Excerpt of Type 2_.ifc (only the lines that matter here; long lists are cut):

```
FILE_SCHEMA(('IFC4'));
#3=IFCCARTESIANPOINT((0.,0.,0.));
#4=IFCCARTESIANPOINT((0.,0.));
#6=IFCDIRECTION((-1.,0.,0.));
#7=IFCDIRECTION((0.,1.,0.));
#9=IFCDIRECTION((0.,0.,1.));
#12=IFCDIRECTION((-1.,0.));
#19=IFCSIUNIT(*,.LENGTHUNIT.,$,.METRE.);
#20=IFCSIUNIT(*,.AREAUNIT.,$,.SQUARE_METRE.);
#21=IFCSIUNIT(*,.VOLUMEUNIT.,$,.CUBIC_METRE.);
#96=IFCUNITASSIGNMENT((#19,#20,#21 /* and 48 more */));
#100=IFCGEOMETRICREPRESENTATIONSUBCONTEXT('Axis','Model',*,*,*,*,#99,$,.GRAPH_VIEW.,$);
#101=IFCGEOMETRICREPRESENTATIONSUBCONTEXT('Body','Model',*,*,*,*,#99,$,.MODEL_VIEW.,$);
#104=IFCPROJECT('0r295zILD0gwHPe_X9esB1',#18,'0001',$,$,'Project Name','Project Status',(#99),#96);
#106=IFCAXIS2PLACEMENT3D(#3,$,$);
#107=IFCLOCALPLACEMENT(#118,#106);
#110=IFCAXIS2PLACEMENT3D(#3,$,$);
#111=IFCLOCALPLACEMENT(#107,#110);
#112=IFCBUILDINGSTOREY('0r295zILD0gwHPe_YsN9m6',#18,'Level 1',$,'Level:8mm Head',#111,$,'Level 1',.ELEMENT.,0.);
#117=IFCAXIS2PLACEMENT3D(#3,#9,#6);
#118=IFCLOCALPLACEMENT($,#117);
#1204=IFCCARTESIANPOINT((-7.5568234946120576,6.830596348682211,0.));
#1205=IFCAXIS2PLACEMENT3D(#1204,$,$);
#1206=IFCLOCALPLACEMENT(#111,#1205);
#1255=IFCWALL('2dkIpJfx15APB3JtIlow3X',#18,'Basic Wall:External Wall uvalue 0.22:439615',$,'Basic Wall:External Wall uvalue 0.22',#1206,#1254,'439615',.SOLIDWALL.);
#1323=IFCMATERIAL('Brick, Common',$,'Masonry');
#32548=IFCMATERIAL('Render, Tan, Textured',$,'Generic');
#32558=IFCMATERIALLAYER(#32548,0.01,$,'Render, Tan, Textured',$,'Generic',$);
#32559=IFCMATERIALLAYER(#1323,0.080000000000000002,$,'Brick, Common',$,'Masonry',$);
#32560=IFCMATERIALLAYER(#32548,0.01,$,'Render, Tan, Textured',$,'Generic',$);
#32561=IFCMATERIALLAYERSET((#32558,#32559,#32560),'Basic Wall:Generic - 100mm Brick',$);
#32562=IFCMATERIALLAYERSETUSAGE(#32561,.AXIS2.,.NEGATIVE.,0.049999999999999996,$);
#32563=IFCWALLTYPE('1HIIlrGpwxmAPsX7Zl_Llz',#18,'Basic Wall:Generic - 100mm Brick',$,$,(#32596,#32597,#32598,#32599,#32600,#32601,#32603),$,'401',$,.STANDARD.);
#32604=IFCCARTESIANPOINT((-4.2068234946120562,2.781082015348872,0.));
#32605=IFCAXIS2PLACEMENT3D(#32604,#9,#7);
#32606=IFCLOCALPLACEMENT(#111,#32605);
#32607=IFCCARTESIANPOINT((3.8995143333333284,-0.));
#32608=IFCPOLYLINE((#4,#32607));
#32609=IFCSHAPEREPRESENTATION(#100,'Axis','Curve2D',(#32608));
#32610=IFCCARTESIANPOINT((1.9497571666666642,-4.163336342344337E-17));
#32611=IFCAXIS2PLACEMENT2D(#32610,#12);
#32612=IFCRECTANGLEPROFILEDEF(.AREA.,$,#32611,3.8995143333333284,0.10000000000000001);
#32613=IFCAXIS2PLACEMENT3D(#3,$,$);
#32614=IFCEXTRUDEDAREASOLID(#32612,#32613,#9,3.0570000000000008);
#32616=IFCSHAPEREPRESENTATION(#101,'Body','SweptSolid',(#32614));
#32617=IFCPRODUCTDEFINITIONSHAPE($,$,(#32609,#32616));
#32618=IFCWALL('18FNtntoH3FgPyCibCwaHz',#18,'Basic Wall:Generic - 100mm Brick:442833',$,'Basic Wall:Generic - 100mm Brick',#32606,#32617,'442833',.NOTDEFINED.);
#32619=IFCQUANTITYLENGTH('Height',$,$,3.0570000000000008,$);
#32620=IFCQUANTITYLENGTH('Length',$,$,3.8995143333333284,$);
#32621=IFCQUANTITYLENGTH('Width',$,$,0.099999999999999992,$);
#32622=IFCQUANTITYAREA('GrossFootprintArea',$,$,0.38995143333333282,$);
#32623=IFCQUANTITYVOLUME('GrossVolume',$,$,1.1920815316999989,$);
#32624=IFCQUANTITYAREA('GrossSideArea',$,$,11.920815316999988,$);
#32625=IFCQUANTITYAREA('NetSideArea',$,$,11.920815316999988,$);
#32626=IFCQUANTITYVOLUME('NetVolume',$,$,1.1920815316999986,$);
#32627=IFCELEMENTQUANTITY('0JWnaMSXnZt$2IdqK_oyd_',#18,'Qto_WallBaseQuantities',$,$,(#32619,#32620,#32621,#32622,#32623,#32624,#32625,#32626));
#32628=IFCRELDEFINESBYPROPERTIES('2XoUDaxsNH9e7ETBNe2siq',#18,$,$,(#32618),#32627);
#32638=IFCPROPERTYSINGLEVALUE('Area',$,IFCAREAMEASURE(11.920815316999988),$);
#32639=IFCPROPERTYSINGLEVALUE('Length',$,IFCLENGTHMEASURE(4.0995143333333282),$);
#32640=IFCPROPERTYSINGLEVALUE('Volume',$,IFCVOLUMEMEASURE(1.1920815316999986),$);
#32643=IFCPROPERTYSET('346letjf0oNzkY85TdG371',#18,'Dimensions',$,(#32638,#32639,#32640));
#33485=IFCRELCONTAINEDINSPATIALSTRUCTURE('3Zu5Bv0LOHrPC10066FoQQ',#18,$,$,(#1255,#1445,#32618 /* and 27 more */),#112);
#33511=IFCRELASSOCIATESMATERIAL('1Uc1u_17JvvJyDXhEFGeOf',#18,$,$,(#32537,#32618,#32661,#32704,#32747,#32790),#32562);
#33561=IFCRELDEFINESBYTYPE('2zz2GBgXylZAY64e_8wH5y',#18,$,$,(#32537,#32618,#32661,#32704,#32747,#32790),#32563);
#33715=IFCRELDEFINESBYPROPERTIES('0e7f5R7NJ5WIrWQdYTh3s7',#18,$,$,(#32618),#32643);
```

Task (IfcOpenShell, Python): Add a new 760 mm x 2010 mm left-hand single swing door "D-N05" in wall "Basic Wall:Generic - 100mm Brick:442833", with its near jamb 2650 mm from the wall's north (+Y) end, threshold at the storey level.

```python
import numpy as np
import ifcopenshell
import ifcopenshell.api.feature
import ifcopenshell.api.geometry
import ifcopenshell.api.pset
import ifcopenshell.api.root
import ifcopenshell.api.spatial
import ifcopenshell.geom
import ifcopenshell.util.element
import ifcopenshell.util.placement
import ifcopenshell.util.representation
import ifcopenshell.util.shape
import ifcopenshell.util.unit

model = ifcopenshell.open("Type 2_.ifc")
unit_scale = ifcopenshell.util.unit.calculate_unit_scale(model)
area_scale = ifcopenshell.util.unit.calculate_unit_scale(model, "AREAUNIT")
volume_scale = ifcopenshell.util.unit.calculate_unit_scale(model, "VOLUMEUNIT")
settings = ifcopenshell.geom.settings()


def volume(element):
    """Net volume in cubic metres, openings subtracted."""
    shape = ifcopenshell.geom.create_shape(settings, element)
    return ifcopenshell.util.shape.get_volume(shape.geometry)


wall = model.by_guid("18FNtntoH3FgPyCibCwaHz")
storey = ifcopenshell.util.element.get_container(wall, ifc_class="IfcBuildingStorey")
context = ifcopenshell.util.representation.get_context(model, "Model", "Body", "MODEL_VIEW")
before = volume(wall)

width, height, from_end, sill = 0.76, 2.01, 2.65, 0.0  # metres

# The wall runs along its own X axis, and the end named is its -X end.
wall_shape = ifcopenshell.geom.create_shape(settings, wall)
x, y, z = ifcopenshell.util.shape.get_vertices(wall_shape.geometry).T
start = x.min() + from_end
face, thickness = float(y.min()), float(y.max() - y.min())
wall_matrix = ifcopenshell.util.placement.get_local_placement(wall.ObjectPlacement)
level = ifcopenshell.util.placement.get_local_placement(storey.ObjectPlacement)[2, 3]


def in_wall(x, y):
    """Placement at x, y metres in the wall's axes, at sill height."""
    matrix = wall_matrix.copy()
    matrix[:, 3] = wall_matrix @ np.array([x / unit_scale, y / unit_scale, 0.0, 1.0])
    matrix[2, 3] = level + sill / unit_scale
    return matrix


# Opening: a box that overshoots both wall faces by 50 mm.
opening = ifcopenshell.api.root.create_entity(model, ifc_class="IfcOpeningElement", predefined_type="OPENING")
box = ifcopenshell.api.geometry.add_wall_representation(
    model, context=context, length=width, height=height, thickness=thickness + 0.1
)
ifcopenshell.api.geometry.assign_representation(model, product=opening, representation=box)
ifcopenshell.api.geometry.edit_object_placement(model, product=opening, matrix=in_wall(start, face - 0.05), is_si=False)
ifcopenshell.api.feature.add_feature(model, feature=opening, element=wall)

door = ifcopenshell.api.root.create_entity(model, ifc_class="IfcDoor", name="D-N05", predefined_type="DOOR")
door.OverallWidth, door.OverallHeight = width / unit_scale, height / unit_scale
door.OperationType = "SINGLE_SWING_LEFT"
body = ifcopenshell.api.geometry.add_door_representation(
    model,
    context=context,
    overall_width=door.OverallWidth,
    overall_height=door.OverallHeight,
    operation_type="SINGLE_SWING_LEFT",
    lining_properties={"LiningDepth": thickness / unit_scale, "ThresholdDepth": thickness / unit_scale},
)
ifcopenshell.api.geometry.assign_representation(model, product=door, representation=body)
ifcopenshell.api.spatial.assign_container(model, products=[door], relating_structure=storey)
ifcopenshell.api.feature.add_filling(model, opening=opening, element=door)

# The lining spans the wall, so the door starts at the wall face.
ifcopenshell.api.geometry.edit_object_placement(model, product=door, matrix=in_wall(start, face), is_si=False)

after = volume(wall)

# Update the wall's stored quantities.
qto = model.by_id(ifcopenshell.util.element.get_pset(wall, "Qto_WallBaseQuantities", should_inherit=False)["id"])
ifcopenshell.api.pset.edit_qto(model, qto=qto, properties={
    "NetSideArea": after / thickness / area_scale,
    "NetVolume": after / volume_scale,
})
pset = model.by_id(ifcopenshell.util.element.get_pset(wall, "Dimensions", should_inherit=False)["id"])
ifcopenshell.api.pset.edit_pset(model, pset=pset, properties={
    "Area": model.create_entity("IfcAreaMeasure", after / thickness / area_scale),
    "Volume": model.create_entity("IfcVolumeMeasure", after / volume_scale),
})

print(f"wall volume {before:.3f} -> {after:.3f} m3")

model.write("Type 2__edited.ifc")
```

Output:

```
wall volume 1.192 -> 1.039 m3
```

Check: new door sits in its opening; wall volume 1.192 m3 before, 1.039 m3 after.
